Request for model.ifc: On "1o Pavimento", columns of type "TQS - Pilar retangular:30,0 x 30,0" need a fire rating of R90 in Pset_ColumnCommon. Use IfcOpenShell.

First a look at what the model holds.

```python
import ifcopenshell
import ifcopenshell.util.element

model = ifcopenshell.open("model.ifc")
print(model.schema)
storey = next(s for s in model.by_type("IfcBuildingStorey") if s.Name == "1o Pavimento")
columns = [e for e in ifcopenshell.util.element.get_decomposition(storey) if e.is_a("IfcColumn")]
seen = {}
for e in columns:
    element_type = ifcopenshell.util.element.get_type(e)
    key = (element_type.Name if element_type != e and element_type else None, ifcopenshell.util.element.get_pset(e, "Pset_ColumnCommon", "FireRating"))
    seen[key] = seen.get(key, 0) + 1
for (name, value), count in sorted(seen.items(), key=str):
    print(count, "x", name, "|", value)
```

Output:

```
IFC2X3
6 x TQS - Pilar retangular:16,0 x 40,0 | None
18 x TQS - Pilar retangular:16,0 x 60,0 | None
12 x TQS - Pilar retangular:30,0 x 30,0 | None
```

```python
import ifcopenshell
import ifcopenshell.api.pset
import ifcopenshell.util.element

model = ifcopenshell.open("model.ifc")

storey = next(s for s in model.by_type("IfcBuildingStorey") if s.Name == "1o Pavimento")
columns = [e for e in ifcopenshell.util.element.get_decomposition(storey) if e.is_a("IfcColumn")]

count = 0
for e in columns:
    element_type = ifcopenshell.util.element.get_type(e)
    if element_type in (None, e) or element_type.Name != "TQS - Pilar retangular:30,0 x 30,0":
        continue
    # add_pset returns the element's existing set when there is one.
    pset = ifcopenshell.api.pset.add_pset(model, product=e, name="Pset_ColumnCommon")
    ifcopenshell.api.pset.edit_pset(model, pset=pset, properties={"FireRating": "R90"})
    count += 1

print(count, "columns updated")

model.write("model_updated.ifc")
```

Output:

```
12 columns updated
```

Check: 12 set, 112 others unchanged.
